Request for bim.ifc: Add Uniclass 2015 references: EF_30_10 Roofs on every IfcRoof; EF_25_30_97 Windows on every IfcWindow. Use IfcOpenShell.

First a look at what the model holds.

```python
import ifcopenshell

model = ifcopenshell.open("bim.ifc")
print(model.schema)
print("classifications:", [c.Name for c in model.by_type("IfcClassification")])
for ifc_class in ("IfcDoor", "IfcRoof", "IfcStair", "IfcWall", "IfcWindow"):
    print(ifc_class, len(model.by_type(ifc_class)))
```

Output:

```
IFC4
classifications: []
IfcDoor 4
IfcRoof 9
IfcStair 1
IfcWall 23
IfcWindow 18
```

```python
import ifcopenshell
import ifcopenshell.api.classification

model = ifcopenshell.open("bim.ifc")

system = ifcopenshell.api.classification.add_classification(model, classification="Uniclass 2015")

codes = {
    "IfcRoof": ("EF_30_10", "Roofs"),
    "IfcWindow": ("EF_25_30_97", "Windows"),
}
for ifc_class, (code, name) in codes.items():
    products = model.by_type(ifc_class)
    ifcopenshell.api.classification.add_reference(
        model, products=products, classification=system, identification=code, name=name
    )
    print(code, len(products))

model.write("bim_v2.ifc")
```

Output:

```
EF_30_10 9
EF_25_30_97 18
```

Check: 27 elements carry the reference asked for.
